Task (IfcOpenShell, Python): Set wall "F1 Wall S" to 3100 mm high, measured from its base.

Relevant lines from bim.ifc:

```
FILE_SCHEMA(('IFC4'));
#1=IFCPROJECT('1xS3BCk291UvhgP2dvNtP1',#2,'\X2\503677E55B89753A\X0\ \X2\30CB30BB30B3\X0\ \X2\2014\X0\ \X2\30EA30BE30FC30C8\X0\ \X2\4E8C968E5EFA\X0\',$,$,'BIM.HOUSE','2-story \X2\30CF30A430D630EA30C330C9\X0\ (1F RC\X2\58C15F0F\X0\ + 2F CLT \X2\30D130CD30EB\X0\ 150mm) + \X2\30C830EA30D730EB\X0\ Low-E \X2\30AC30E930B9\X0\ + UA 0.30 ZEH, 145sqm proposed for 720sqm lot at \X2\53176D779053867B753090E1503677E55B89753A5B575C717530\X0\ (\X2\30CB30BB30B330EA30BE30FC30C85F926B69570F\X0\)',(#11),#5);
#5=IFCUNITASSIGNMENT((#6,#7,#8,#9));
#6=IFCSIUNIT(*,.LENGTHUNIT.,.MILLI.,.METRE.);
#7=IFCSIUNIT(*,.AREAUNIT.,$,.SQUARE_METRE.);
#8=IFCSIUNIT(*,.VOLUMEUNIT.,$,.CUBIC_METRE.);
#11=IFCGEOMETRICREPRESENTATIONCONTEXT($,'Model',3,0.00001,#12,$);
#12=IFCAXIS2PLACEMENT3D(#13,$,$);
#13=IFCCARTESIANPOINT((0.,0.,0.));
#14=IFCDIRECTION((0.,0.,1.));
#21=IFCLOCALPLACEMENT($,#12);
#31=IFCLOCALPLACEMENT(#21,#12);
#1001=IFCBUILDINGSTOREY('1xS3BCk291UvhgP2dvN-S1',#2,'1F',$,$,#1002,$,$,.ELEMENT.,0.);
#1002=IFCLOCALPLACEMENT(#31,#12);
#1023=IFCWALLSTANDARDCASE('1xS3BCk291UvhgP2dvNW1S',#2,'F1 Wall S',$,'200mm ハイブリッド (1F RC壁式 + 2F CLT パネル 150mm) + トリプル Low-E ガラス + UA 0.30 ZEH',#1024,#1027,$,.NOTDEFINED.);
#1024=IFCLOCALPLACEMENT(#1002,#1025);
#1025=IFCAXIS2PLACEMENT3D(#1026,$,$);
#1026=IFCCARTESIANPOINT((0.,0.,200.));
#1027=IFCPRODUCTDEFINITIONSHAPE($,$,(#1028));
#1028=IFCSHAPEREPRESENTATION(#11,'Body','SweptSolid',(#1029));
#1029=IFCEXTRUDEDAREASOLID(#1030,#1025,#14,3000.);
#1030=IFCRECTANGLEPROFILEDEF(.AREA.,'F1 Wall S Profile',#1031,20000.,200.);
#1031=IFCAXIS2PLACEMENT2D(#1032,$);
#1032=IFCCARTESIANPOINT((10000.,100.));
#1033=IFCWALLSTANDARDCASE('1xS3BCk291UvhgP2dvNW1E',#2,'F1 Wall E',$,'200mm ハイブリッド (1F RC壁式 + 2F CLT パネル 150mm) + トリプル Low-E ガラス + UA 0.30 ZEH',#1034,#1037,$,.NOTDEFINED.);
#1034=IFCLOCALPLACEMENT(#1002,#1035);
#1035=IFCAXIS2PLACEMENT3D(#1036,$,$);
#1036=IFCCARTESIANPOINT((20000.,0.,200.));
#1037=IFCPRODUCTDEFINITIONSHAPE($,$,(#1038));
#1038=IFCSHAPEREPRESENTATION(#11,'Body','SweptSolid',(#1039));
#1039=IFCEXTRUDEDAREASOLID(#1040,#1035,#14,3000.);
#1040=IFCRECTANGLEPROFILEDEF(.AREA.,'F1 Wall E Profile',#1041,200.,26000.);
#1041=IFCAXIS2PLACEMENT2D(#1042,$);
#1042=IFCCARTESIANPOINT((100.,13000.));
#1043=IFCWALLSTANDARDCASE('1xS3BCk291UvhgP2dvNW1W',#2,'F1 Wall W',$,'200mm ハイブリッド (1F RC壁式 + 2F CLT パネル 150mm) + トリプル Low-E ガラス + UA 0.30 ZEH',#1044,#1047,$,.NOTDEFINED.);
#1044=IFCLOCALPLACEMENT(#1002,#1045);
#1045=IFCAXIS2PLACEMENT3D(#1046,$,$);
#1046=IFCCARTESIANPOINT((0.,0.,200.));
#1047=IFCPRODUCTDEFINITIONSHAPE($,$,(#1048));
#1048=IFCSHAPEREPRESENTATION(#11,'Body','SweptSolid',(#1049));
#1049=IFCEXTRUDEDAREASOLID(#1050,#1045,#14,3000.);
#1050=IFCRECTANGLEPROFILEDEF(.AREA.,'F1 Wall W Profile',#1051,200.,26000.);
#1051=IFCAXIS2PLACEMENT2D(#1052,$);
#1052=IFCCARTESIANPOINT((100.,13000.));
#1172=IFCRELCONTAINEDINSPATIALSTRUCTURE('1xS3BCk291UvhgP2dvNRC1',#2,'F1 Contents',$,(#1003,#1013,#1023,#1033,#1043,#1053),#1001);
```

```python
import ifcopenshell
import ifcopenshell.geom
import ifcopenshell.util.shape

model = ifcopenshell.open("bim.ifc")
settings = ifcopenshell.geom.settings()


def volume(element):
    """Net volume in cubic metres, openings subtracted."""
    shape = ifcopenshell.geom.create_shape(settings, element)
    return ifcopenshell.util.shape.get_volume(shape.geometry)


wall = model.by_id(1023)
before = volume(wall)

body = next(r for r in wall.Representation.Representations if r.RepresentationIdentifier == "Body")
solid = body.Items[0]
old_height = solid.Depth
solid.Depth = 3100.0
after = volume(wall)

print(f"height {old_height:g} -> {solid.Depth:g}, volume {before:.3f} -> {after:.3f} m3")

model.write("bim_rev.ifc")
```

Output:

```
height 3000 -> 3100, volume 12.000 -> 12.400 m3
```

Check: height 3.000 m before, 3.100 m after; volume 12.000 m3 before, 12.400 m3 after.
